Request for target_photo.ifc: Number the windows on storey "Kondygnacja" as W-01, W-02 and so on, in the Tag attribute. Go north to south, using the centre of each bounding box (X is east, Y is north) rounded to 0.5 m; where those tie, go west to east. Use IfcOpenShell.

First a look at what the model holds.

```python
import ifcopenshell
import ifcopenshell.util.element
import ifcopenshell.util.placement

model = ifcopenshell.open("target_photo.ifc")
print(model.schema)
storey = next(s for s in model.by_type("IfcBuildingStorey") if s.Name == "Kondygnacja")
windows = [e for e in ifcopenshell.util.element.get_decomposition(storey) if e.is_a("IfcWindow")]
for e in sorted(windows, key=lambda e: e.id()):
    origin = ifcopenshell.util.placement.get_local_placement(e.ObjectPlacement)[:3, 3]
    print(e.id(), e.Tag, e.Name, origin.round(2) + 0.0, sep=" | ")
```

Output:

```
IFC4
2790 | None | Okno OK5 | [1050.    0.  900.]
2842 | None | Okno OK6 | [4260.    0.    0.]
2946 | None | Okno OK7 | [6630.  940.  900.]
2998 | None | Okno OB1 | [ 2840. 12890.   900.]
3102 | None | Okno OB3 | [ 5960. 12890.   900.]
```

```python
import ifcopenshell
import ifcopenshell.geom
import ifcopenshell.util.element
import ifcopenshell.util.shape

model = ifcopenshell.open("target_photo.ifc")
settings = ifcopenshell.geom.settings()
settings.set("use-world-coords", True)


def centre(element):
    shape = ifcopenshell.geom.create_shape(settings, element)
    return ifcopenshell.util.shape.get_bbox_centroid(shape.geometry)


storey = next(s for s in model.by_type("IfcBuildingStorey") if s.Name == "Kondygnacja")
windows = [e for e in ifcopenshell.util.element.get_decomposition(storey) if e.is_a("IfcWindow")]

# Insertion points can sit at a corner or the storey origin, so sort by the geometry (in metres).
centres = {e: centre(e) for e in windows}
windows.sort(key=lambda e: (-round(centres[e][1] / 0.5), centres[e][0]))

for i, e in enumerate(windows, start=1):
    number = f"W-{i:02d}"
    e.Tag = number
    print(e.id(), number)

model.write("target_photo_updated.ifc")
```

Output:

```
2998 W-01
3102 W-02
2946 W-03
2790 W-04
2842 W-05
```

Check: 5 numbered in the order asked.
